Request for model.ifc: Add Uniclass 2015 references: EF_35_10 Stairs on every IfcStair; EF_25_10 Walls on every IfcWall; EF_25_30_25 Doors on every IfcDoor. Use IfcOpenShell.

First a look at what the model holds.

```python
import ifcopenshell

model = ifcopenshell.open("model.ifc")
print(model.schema)
print("classifications:", [c.Name for c in model.by_type("IfcClassification")])
for ifc_class in ("IfcDoor", "IfcRoof", "IfcStair", "IfcWall", "IfcWindow"):
    print(ifc_class, len(model.by_type(ifc_class)))
```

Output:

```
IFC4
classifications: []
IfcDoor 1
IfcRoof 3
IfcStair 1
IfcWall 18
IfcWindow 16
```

```python
import ifcopenshell
import ifcopenshell.api.classification

model = ifcopenshell.open("model.ifc")

system = ifcopenshell.api.classification.add_classification(model, classification="Uniclass 2015")

codes = {
    "IfcStair": ("EF_35_10", "Stairs"),
    "IfcWall": ("EF_25_10", "Walls"),
    "IfcDoor": ("EF_25_30_25", "Doors"),
}
for ifc_class, (code, name) in codes.items():
    products = model.by_type(ifc_class)
    ifcopenshell.api.classification.add_reference(
        model, products=products, classification=system, identification=code, name=name
    )
    print(code, len(products))

model.write("model_rev.ifc")
```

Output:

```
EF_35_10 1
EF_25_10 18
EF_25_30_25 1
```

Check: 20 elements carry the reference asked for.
